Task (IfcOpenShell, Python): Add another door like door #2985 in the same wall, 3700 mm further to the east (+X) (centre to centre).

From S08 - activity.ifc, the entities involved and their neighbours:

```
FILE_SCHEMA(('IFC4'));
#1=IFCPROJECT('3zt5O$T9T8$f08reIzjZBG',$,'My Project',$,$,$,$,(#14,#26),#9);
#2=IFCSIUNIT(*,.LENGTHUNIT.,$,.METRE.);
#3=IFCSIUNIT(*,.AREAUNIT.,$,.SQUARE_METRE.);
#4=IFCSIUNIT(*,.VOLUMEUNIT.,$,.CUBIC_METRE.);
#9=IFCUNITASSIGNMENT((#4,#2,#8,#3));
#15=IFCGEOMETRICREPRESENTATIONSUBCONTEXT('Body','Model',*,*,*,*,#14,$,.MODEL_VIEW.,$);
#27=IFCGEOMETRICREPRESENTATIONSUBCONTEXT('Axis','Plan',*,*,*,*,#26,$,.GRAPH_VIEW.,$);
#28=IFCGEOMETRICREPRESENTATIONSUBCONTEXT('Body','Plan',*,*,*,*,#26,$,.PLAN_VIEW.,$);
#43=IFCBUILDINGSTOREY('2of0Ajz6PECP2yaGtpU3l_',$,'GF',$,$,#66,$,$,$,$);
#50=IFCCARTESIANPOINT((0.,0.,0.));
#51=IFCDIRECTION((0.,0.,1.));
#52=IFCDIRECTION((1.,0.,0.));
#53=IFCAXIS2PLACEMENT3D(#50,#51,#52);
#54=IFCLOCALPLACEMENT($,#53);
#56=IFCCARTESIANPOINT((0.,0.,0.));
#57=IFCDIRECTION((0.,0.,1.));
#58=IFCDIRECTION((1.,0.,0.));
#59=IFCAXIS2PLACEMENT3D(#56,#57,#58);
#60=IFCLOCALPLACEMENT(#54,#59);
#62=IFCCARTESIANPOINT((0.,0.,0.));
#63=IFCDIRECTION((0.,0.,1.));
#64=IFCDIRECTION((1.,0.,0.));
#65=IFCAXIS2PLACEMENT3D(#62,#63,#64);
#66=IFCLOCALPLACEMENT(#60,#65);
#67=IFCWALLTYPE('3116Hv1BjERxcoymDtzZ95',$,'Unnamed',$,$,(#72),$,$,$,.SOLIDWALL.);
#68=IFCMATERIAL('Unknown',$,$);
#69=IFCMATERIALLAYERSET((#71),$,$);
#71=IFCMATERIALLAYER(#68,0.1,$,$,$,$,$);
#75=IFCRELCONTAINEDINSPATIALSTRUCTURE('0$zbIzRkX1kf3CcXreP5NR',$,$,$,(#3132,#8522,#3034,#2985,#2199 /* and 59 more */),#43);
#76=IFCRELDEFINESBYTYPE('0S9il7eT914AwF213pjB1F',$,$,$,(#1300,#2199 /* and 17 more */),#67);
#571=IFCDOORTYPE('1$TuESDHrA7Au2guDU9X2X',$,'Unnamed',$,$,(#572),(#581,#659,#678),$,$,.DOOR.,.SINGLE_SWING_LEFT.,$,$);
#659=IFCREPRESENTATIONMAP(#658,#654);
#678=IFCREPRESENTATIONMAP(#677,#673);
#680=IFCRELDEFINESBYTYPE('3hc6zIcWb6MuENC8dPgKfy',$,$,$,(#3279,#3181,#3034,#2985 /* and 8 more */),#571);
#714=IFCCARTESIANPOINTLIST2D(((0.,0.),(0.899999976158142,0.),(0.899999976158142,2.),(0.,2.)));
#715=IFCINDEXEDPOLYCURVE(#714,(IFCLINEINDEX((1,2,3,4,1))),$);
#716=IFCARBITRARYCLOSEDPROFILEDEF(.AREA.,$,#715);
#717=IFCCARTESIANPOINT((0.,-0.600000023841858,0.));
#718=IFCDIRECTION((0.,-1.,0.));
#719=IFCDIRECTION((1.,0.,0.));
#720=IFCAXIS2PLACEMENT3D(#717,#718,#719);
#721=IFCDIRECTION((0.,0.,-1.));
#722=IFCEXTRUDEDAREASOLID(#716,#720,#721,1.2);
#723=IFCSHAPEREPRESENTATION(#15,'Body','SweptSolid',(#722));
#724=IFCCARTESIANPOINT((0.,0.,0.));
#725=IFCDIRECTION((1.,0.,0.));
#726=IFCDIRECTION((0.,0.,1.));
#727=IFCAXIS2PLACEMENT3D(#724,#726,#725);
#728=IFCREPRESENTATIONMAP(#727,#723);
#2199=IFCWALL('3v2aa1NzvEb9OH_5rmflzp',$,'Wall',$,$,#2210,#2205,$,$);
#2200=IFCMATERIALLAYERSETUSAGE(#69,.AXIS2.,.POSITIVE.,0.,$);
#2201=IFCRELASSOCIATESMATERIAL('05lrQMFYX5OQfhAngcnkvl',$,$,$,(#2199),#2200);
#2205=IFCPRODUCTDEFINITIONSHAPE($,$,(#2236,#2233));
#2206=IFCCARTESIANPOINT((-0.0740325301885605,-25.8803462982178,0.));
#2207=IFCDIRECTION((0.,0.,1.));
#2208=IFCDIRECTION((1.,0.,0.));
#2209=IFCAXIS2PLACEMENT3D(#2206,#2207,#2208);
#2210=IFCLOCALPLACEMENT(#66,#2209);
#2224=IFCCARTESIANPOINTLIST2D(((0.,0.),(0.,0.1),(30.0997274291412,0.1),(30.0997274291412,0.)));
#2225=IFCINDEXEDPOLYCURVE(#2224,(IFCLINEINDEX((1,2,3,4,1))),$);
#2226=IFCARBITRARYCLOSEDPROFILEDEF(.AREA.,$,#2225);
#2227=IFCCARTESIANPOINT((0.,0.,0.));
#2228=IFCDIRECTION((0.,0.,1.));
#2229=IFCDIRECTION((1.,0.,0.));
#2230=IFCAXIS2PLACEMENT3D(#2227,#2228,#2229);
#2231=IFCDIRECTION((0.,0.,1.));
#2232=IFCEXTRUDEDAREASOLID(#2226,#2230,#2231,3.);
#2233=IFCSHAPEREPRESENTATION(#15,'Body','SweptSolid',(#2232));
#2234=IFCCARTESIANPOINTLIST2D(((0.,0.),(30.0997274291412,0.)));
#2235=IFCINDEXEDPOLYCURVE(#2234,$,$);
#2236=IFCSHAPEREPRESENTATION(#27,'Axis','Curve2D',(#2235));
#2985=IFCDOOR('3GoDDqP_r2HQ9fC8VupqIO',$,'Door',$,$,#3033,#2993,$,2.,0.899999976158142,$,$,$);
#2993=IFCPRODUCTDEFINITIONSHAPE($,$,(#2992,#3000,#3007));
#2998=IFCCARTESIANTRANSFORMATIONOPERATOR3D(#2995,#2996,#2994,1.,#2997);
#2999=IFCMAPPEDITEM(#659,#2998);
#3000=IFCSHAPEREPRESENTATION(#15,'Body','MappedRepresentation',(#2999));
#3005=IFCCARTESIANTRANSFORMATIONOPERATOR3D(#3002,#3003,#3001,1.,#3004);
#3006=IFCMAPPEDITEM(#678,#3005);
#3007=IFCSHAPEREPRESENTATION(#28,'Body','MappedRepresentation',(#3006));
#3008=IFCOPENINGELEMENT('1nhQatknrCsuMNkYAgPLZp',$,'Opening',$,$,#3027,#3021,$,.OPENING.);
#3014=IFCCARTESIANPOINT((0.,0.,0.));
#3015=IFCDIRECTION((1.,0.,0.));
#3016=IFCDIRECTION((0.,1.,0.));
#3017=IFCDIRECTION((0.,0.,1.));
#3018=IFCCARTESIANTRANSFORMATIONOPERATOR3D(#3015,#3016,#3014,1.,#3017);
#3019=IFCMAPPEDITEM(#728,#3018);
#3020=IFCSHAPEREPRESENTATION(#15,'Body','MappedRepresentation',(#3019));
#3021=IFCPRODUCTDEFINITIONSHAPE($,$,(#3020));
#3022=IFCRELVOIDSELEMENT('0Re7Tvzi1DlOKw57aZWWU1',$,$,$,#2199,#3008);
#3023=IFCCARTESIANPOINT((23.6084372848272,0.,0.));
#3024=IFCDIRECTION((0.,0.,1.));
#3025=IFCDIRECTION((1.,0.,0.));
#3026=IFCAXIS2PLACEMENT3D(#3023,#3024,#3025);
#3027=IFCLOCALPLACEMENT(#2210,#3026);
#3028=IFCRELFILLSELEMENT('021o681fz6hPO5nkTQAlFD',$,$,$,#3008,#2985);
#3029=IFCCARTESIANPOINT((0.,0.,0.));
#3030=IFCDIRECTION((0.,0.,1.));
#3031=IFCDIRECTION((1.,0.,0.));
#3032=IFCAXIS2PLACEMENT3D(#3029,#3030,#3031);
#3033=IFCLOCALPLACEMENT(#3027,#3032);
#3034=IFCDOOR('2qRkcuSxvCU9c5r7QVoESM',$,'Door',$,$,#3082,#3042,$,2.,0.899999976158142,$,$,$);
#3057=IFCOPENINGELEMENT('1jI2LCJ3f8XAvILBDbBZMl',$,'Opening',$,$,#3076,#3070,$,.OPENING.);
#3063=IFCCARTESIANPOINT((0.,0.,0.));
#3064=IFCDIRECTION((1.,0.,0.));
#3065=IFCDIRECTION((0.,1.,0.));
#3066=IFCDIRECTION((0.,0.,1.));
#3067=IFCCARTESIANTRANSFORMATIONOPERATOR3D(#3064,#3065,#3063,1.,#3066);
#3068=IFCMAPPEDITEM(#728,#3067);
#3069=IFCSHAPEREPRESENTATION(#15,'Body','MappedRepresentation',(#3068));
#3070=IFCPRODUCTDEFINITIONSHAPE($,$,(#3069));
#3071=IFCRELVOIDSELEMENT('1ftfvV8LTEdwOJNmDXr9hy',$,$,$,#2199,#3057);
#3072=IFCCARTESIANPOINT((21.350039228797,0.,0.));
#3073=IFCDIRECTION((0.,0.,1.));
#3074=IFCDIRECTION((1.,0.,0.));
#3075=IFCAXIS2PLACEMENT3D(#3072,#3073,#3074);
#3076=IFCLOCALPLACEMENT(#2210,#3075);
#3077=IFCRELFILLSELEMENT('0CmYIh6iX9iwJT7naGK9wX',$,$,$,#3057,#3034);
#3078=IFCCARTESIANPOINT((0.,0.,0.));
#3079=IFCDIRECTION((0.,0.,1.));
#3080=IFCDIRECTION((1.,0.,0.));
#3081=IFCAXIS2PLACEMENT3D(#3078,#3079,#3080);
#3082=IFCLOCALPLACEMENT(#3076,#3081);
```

```python
import ifcopenshell
import ifcopenshell.api.feature
import ifcopenshell.api.geometry
import ifcopenshell.api.root
import ifcopenshell.geom
import ifcopenshell.util.element
import ifcopenshell.util.placement
import ifcopenshell.util.shape

model = ifcopenshell.open("S08 - activity.ifc")
settings = ifcopenshell.geom.settings()


def volume(element):
    """Net volume in cubic metres, openings subtracted."""
    shape = ifcopenshell.geom.create_shape(settings, element)
    return ifcopenshell.util.shape.get_volume(shape.geometry)


door = model.by_guid("3GoDDqP_r2HQ9fC8VupqIO")
opening = door.FillsVoids[0].RelatingOpeningElement
wall = opening.VoidsElements[0].RelatingBuildingElement
before = volume(wall)
shift = ifcopenshell.util.placement.get_local_placement(wall.ObjectPlacement)[:3, 0] * 3.7

# copy_class copies the void relationship, type, container and properties, but no geometry.
new_opening = ifcopenshell.api.root.copy_class(model, product=opening)
new_opening.Representation = ifcopenshell.util.element.copy_deep(
    model, opening.Representation, exclude=["IfcGeometricRepresentationContext", "IfcRepresentationMap"]
)
new_door = ifcopenshell.api.root.copy_class(model, product=door)
new_door.Representation = ifcopenshell.util.element.copy_deep(
    model, door.Representation, exclude=["IfcGeometricRepresentationContext", "IfcRepresentationMap"]
)
ifcopenshell.api.feature.add_filling(model, opening=new_opening, element=new_door)

for old, new in ((opening, new_opening), (door, new_door)):
    matrix = ifcopenshell.util.placement.get_local_placement(old.ObjectPlacement)
    matrix[:3, 3] += shift
    ifcopenshell.api.geometry.edit_object_placement(model, product=new, matrix=matrix, is_si=False)

after = volume(wall)

print(f"wall volume {before:.3f} -> {after:.3f} m3")

model.write("S08 - activity_edited.ifc")
```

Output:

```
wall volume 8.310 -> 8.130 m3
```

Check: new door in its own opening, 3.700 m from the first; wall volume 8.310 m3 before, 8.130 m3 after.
